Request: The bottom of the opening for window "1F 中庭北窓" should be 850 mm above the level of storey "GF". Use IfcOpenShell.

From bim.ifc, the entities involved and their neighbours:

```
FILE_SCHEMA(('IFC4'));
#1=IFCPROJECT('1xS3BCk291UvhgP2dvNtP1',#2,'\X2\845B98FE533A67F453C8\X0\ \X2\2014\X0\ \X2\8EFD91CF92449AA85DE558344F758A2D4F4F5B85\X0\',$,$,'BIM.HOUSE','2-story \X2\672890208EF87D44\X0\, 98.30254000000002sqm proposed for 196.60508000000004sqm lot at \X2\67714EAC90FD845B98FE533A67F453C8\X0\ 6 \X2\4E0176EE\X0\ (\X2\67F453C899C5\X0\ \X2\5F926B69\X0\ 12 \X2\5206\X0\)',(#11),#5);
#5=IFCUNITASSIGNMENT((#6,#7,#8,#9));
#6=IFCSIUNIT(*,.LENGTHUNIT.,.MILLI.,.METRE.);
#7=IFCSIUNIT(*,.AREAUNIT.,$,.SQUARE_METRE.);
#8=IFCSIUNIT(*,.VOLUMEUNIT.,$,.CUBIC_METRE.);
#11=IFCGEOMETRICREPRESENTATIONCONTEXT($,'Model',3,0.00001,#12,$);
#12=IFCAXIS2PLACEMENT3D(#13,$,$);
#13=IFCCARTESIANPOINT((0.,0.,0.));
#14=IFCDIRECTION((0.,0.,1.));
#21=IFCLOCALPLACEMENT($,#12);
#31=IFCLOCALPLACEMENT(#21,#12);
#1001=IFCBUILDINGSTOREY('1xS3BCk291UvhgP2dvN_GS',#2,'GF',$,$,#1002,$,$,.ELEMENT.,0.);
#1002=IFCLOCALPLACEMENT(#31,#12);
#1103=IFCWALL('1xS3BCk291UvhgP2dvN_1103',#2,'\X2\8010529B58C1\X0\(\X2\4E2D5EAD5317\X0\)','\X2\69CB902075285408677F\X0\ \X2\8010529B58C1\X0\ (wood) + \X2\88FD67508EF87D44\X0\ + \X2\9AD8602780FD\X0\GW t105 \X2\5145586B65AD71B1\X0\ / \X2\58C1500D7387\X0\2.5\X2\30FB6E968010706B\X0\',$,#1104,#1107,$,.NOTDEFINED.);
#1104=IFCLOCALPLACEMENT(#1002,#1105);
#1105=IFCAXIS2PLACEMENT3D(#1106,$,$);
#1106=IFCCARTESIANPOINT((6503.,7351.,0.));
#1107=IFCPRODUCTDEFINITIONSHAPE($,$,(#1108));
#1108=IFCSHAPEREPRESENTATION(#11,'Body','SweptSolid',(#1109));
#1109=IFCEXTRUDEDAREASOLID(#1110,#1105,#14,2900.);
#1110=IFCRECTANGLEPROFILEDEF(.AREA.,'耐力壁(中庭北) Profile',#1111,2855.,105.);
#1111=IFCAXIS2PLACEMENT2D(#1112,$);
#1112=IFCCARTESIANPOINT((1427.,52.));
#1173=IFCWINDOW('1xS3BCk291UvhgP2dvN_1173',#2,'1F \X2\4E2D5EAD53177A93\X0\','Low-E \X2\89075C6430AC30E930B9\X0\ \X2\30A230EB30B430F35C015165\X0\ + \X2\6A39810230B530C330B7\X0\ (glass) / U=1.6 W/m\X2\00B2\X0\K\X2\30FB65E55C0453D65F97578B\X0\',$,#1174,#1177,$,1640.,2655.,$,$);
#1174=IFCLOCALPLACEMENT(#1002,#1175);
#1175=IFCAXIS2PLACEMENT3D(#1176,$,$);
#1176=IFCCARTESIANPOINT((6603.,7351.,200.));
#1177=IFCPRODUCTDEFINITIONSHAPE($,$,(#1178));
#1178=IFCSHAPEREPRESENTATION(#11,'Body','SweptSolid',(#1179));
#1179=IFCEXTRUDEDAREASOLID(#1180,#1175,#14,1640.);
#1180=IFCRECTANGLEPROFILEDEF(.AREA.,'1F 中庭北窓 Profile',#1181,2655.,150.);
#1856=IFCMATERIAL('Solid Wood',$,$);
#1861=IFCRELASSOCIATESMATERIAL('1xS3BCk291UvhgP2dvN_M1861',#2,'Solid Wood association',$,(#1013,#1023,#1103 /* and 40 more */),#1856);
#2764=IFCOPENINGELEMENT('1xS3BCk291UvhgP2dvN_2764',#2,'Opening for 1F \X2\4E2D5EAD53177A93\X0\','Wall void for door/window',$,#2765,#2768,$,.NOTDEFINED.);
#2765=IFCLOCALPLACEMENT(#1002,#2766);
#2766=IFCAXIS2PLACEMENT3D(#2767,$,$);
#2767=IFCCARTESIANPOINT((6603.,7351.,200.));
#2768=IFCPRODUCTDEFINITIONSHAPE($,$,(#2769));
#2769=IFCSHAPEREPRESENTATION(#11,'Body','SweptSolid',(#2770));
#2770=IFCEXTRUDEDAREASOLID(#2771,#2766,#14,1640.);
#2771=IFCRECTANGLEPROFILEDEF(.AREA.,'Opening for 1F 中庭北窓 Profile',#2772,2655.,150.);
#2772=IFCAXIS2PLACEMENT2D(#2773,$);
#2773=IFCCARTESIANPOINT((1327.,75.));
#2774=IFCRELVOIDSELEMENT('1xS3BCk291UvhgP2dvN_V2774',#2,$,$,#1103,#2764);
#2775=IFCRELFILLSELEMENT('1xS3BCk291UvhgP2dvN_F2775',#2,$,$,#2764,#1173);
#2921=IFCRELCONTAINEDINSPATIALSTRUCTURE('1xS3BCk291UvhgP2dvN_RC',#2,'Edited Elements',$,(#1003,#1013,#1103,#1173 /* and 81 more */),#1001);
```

```python
import numpy as np
import ifcopenshell
import ifcopenshell.api.geometry
import ifcopenshell.geom
import ifcopenshell.util.element
import ifcopenshell.util.placement
import ifcopenshell.util.shape
import ifcopenshell.util.unit

model = ifcopenshell.open("bim.ifc")
unit_scale = ifcopenshell.util.unit.calculate_unit_scale(model)

window = model.by_guid("1xS3BCk291UvhgP2dvN_1173")
opening = window.FillsVoids[0].RelatingOpeningElement
storey = ifcopenshell.util.element.get_container(window, ifc_class="IfcBuildingStorey")
level = ifcopenshell.util.placement.get_local_placement(storey.ObjectPlacement)[2, 3]

# The opening's origin need not be at the sill, so measure its lowest point.
shape = ifcopenshell.geom.create_shape(ifcopenshell.geom.settings(), opening)
bottom = ifcopenshell.util.shape.get_shape_bottom_elevation(shape, shape.geometry) / unit_scale
dz = level + 850.0 - bottom

shift = np.array([0.0, 0.0, dz])
# The window is not placed relative to its opening, so move both.
for product in (opening, window):
    matrix = ifcopenshell.util.placement.get_local_placement(product.ObjectPlacement)
    matrix[:3, 3] += shift
    ifcopenshell.api.geometry.edit_object_placement(model, product=product, matrix=matrix, is_si=False)

print(f"moved by {dz * unit_scale:+.3f} m")

model.write("bim_edited.ifc")
```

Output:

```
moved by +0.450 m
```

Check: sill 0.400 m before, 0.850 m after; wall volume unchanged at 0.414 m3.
